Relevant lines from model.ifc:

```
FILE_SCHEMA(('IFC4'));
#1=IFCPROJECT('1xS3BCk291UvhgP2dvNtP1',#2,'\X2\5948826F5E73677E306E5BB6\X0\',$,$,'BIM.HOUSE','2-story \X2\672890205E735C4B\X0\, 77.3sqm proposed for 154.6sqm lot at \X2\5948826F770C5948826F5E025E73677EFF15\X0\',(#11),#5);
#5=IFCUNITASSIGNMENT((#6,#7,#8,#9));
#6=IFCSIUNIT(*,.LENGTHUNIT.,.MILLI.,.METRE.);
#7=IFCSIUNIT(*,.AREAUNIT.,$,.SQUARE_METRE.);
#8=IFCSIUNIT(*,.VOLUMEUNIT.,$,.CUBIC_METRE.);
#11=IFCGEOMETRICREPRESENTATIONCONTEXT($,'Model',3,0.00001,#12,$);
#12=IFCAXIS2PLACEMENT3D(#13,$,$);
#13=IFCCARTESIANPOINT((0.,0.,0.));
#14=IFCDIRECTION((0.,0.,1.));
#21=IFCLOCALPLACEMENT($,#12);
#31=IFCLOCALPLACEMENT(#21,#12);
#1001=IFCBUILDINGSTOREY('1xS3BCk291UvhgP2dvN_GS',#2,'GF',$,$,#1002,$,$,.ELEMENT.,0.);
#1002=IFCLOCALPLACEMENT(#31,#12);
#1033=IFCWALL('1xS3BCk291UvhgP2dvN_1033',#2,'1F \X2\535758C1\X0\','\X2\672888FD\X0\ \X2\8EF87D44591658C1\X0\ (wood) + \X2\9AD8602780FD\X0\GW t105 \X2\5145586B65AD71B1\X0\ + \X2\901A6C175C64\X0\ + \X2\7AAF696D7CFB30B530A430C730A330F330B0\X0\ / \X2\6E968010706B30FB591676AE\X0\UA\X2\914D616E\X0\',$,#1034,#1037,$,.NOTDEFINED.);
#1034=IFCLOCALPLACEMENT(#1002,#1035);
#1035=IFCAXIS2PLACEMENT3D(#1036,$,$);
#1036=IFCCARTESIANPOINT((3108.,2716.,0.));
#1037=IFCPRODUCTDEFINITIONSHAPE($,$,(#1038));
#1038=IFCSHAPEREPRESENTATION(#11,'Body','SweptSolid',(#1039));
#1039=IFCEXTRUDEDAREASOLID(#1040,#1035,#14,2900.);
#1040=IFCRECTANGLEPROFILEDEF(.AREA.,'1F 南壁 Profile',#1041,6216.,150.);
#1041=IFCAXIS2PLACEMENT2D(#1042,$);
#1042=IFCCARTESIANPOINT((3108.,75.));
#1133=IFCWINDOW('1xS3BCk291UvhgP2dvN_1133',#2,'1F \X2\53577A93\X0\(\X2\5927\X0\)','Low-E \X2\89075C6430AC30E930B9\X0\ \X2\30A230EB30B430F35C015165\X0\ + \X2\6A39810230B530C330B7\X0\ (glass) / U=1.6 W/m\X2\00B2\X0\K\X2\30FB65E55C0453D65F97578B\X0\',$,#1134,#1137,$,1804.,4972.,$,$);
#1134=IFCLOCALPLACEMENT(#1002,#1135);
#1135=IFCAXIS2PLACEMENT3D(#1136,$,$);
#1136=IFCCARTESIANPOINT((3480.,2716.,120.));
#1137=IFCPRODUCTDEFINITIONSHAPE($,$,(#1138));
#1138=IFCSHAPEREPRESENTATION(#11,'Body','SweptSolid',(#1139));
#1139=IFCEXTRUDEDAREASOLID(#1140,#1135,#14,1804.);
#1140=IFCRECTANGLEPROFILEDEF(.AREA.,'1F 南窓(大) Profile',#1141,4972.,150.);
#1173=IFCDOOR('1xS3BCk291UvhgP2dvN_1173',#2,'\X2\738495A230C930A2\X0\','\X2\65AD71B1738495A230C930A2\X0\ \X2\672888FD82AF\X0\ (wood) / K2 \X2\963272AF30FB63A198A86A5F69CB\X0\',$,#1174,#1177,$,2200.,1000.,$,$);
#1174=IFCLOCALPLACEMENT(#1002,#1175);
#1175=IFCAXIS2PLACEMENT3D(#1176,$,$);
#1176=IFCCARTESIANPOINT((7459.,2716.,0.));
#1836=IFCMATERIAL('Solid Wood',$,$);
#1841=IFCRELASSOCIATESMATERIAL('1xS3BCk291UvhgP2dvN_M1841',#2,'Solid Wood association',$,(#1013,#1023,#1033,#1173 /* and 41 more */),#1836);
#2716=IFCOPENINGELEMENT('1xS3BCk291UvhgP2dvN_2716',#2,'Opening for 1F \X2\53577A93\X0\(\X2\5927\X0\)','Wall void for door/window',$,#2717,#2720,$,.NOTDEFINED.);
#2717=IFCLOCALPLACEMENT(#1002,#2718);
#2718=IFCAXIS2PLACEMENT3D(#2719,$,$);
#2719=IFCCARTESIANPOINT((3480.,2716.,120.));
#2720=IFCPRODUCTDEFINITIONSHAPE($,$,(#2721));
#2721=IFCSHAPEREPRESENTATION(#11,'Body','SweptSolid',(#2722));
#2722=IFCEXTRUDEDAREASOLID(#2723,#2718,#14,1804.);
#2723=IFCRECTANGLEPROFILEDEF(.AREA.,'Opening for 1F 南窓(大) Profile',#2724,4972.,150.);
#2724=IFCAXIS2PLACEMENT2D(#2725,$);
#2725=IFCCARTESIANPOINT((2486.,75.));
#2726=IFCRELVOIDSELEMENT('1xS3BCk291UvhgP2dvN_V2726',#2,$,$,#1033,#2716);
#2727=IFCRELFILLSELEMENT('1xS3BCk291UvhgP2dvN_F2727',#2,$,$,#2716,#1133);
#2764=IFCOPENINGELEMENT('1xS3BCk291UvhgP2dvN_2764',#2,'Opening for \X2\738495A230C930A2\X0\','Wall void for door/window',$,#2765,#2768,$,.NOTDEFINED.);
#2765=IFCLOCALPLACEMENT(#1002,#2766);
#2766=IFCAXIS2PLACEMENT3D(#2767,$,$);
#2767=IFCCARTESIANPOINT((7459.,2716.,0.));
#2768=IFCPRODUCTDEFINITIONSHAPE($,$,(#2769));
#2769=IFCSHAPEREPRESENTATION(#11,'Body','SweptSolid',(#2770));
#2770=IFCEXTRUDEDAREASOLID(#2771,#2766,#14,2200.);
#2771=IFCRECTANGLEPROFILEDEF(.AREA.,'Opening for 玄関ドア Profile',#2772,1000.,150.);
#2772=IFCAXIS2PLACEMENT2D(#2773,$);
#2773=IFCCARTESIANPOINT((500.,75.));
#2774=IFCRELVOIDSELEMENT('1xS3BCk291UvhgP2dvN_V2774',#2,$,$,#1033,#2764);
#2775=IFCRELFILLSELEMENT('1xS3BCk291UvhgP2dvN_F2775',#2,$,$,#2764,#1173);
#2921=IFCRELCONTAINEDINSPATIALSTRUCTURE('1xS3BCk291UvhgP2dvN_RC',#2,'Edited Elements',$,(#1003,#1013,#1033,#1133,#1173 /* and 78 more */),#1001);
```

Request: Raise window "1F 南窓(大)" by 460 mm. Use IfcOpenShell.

```python
import numpy as np
import ifcopenshell
import ifcopenshell.api.geometry
import ifcopenshell.util.placement
import ifcopenshell.util.unit

model = ifcopenshell.open("model.ifc")
unit_scale = ifcopenshell.util.unit.calculate_unit_scale(model)

window = model.by_id(1133)
opening = window.FillsVoids[0].RelatingOpeningElement
dz = 0.46 / unit_scale

shift = np.array([0.0, 0.0, dz])
# The window is not placed relative to its opening, so move both.
for product in (opening, window):
    matrix = ifcopenshell.util.placement.get_local_placement(product.ObjectPlacement)
    matrix[:3, 3] += shift
    ifcopenshell.api.geometry.edit_object_placement(model, product=product, matrix=matrix, is_si=False)

print(f"moved by {dz * unit_scale:+.3f} m")

model.write("model-out.ifc")
```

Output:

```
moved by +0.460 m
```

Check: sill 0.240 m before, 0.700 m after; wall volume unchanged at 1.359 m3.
